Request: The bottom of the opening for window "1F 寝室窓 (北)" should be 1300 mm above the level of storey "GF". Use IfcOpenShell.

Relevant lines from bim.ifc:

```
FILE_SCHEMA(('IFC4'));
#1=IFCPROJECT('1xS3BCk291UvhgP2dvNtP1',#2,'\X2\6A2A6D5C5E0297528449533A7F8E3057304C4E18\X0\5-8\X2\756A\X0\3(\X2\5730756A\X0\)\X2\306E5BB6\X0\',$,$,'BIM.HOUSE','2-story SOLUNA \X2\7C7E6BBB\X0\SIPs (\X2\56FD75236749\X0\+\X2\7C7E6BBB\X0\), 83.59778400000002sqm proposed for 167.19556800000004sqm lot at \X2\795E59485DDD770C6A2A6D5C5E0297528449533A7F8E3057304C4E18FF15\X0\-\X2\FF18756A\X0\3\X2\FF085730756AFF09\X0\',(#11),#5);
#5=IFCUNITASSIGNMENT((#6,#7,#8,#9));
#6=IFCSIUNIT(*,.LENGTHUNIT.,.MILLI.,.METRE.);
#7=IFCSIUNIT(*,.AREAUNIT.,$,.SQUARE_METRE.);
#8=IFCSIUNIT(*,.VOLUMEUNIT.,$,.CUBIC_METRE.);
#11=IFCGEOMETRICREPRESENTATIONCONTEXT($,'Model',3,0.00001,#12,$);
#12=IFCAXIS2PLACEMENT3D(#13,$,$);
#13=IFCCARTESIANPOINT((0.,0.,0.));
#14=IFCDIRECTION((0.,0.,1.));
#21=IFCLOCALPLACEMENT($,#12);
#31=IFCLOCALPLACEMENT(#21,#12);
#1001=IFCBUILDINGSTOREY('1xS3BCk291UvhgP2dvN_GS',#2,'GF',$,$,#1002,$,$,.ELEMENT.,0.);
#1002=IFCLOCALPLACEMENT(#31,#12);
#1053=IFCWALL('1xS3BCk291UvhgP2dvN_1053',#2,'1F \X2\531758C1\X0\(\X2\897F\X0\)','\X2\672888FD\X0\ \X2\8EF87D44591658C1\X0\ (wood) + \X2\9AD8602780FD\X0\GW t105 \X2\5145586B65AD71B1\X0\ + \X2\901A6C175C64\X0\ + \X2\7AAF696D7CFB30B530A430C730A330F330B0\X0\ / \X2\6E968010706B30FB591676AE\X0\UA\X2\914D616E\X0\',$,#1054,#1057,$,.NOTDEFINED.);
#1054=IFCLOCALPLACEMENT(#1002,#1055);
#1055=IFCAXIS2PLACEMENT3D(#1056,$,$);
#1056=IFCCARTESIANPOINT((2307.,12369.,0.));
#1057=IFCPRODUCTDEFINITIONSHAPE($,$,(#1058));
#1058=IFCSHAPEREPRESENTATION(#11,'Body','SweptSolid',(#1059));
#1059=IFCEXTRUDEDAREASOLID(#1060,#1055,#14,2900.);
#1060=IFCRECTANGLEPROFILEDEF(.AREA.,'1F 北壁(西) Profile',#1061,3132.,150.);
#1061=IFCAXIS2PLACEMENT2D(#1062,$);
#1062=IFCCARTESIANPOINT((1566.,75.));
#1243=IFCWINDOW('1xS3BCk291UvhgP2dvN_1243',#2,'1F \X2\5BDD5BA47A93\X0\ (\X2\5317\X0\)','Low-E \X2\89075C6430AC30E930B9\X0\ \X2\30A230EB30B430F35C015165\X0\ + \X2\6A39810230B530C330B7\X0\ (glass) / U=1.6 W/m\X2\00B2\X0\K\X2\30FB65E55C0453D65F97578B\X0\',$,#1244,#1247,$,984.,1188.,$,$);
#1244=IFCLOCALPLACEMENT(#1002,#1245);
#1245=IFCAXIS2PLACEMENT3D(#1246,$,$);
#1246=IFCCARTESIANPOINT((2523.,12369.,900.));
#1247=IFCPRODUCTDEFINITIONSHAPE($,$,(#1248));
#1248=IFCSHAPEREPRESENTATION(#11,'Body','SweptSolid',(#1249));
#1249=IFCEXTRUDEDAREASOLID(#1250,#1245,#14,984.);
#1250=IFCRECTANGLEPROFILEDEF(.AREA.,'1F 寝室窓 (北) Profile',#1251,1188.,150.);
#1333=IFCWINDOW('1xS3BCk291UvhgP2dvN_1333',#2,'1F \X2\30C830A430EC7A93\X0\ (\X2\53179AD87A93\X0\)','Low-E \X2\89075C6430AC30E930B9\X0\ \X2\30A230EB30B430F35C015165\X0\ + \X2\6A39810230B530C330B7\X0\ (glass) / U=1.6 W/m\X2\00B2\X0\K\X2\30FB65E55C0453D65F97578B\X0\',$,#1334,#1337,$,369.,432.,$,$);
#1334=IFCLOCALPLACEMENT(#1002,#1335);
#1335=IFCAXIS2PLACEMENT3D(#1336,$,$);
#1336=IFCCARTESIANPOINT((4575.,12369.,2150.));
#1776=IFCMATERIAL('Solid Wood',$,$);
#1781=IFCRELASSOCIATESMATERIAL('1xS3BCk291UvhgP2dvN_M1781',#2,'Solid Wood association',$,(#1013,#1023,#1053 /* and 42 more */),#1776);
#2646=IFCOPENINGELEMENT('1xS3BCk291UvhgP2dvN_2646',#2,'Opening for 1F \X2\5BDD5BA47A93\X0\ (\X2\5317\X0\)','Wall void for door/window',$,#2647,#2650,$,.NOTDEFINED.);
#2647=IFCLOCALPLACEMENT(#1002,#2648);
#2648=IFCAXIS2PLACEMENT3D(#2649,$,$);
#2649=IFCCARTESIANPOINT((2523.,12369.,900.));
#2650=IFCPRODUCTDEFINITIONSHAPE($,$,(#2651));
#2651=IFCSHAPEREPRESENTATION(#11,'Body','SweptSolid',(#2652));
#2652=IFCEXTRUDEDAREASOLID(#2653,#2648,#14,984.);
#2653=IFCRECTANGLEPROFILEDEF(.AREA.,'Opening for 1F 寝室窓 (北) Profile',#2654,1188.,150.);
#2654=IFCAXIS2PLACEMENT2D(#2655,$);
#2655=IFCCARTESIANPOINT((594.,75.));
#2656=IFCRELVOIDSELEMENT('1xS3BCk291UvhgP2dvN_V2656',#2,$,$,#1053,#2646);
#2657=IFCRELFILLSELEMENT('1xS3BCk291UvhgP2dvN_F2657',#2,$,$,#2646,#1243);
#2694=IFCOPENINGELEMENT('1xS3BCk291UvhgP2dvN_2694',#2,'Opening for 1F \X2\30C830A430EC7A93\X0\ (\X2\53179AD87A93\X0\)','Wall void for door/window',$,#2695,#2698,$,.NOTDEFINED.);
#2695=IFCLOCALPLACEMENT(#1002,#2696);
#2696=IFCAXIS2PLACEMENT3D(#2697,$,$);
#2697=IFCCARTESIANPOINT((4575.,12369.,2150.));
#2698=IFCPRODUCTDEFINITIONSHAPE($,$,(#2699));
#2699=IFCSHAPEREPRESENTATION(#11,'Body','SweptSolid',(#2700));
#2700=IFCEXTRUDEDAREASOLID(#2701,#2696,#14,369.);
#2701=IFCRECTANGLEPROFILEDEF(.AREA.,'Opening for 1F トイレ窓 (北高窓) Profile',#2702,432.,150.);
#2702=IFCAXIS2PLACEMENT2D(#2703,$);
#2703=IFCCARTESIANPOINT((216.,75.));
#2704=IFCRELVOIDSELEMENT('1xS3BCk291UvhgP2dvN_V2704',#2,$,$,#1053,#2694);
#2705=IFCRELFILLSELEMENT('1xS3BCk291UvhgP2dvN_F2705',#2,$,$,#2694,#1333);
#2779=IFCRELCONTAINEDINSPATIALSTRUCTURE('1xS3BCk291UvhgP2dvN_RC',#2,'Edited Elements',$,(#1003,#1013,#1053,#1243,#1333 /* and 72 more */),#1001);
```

```python
import numpy as np
import ifcopenshell
import ifcopenshell.api.geometry
import ifcopenshell.geom
import ifcopenshell.util.element
import ifcopenshell.util.placement
import ifcopenshell.util.shape
import ifcopenshell.util.unit

model = ifcopenshell.open("bim.ifc")
unit_scale = ifcopenshell.util.unit.calculate_unit_scale(model)

window = model.by_guid("1xS3BCk291UvhgP2dvN_1243")
opening = window.FillsVoids[0].RelatingOpeningElement
storey = ifcopenshell.util.element.get_container(window, ifc_class="IfcBuildingStorey")
level = ifcopenshell.util.placement.get_local_placement(storey.ObjectPlacement)[2, 3]

# The opening's origin need not be at the sill, so measure its lowest point.
shape = ifcopenshell.geom.create_shape(ifcopenshell.geom.settings(), opening)
bottom = ifcopenshell.util.shape.get_shape_bottom_elevation(shape, shape.geometry) / unit_scale
dz = level + 1.3 / unit_scale - bottom

shift = np.array([0.0, 0.0, dz])
# The window is not placed relative to its opening, so move both.
for product in (opening, window):
    matrix = ifcopenshell.util.placement.get_local_placement(product.ObjectPlacement)
    matrix[:3, 3] += shift
    ifcopenshell.api.geometry.edit_object_placement(model, product=product, matrix=matrix, is_si=False)

print(f"moved by {dz * unit_scale:+.3f} m")

model.write("bim_rev.ifc")
```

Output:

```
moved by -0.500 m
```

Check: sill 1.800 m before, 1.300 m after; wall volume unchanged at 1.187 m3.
